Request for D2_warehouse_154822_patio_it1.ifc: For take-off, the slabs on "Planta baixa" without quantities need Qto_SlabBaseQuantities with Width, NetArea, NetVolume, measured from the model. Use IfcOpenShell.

First a look at what the model holds.

```python
import ifcopenshell
import ifcopenshell.util.element
import ifcopenshell.util.unit

model = ifcopenshell.open("D2_warehouse_154822_patio_it1.ifc")
print(model.schema)
for unit_type in ("LENGTHUNIT", "AREAUNIT", "VOLUMEUNIT"):
    print(unit_type, ifcopenshell.util.unit.calculate_unit_scale(model, unit_type))
storey = next(s for s in model.by_type("IfcBuildingStorey") if s.Name == "Planta baixa")
slabs = [e for e in ifcopenshell.util.element.get_decomposition(storey) if e.is_a("IfcSlab")]
for e in sorted(slabs, key=lambda e: e.id()):
    print(e.id(), e.is_a(), e.Name, list(ifcopenshell.util.element.get_psets(e, qtos_only=True)), sep=" | ")
```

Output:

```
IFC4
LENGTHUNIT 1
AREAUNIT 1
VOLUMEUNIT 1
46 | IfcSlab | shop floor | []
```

```python
import ifcopenshell
import ifcopenshell.api.pset
import ifcopenshell.geom
import ifcopenshell.util.element
import ifcopenshell.util.shape
import ifcopenshell.util.unit

model = ifcopenshell.open("D2_warehouse_154822_patio_it1.ifc")
unit_scale = ifcopenshell.util.unit.calculate_unit_scale(model)
area_scale = ifcopenshell.util.unit.calculate_unit_scale(model, "AREAUNIT")
volume_scale = ifcopenshell.util.unit.calculate_unit_scale(model, "VOLUMEUNIT")
settings = ifcopenshell.geom.settings()

storey = next(s for s in model.by_type("IfcBuildingStorey") if s.Name == "Planta baixa")
slabs = [e for e in ifcopenshell.util.element.get_decomposition(storey) if e.is_a("IfcSlab")]

for e in sorted(slabs, key=lambda e: e.id()):
    if ifcopenshell.util.element.get_psets(e, qtos_only=True, should_inherit=False):
        continue
    # Geometry comes back in metres, in the element's own axes.
    shape = ifcopenshell.geom.create_shape(settings, e)
    values = {
        "Width": ifcopenshell.util.shape.get_z(shape.geometry) / unit_scale,
        "NetArea": ifcopenshell.util.shape.get_footprint_area(shape.geometry) / area_scale,
        "NetVolume": ifcopenshell.util.shape.get_volume(shape.geometry) / volume_scale,
    }
    qto = ifcopenshell.api.pset.add_qto(model, product=e, name="Qto_SlabBaseQuantities")
    ifcopenshell.api.pset.edit_qto(model, qto=qto, properties=values)
    print(e.id(), {k: round(v, 3) for k, v in values.items()})

model.write("D2_warehouse_154822_patio_it1_edited.ifc")
```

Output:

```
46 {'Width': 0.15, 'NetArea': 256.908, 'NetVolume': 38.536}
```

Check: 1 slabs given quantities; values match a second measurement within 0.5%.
